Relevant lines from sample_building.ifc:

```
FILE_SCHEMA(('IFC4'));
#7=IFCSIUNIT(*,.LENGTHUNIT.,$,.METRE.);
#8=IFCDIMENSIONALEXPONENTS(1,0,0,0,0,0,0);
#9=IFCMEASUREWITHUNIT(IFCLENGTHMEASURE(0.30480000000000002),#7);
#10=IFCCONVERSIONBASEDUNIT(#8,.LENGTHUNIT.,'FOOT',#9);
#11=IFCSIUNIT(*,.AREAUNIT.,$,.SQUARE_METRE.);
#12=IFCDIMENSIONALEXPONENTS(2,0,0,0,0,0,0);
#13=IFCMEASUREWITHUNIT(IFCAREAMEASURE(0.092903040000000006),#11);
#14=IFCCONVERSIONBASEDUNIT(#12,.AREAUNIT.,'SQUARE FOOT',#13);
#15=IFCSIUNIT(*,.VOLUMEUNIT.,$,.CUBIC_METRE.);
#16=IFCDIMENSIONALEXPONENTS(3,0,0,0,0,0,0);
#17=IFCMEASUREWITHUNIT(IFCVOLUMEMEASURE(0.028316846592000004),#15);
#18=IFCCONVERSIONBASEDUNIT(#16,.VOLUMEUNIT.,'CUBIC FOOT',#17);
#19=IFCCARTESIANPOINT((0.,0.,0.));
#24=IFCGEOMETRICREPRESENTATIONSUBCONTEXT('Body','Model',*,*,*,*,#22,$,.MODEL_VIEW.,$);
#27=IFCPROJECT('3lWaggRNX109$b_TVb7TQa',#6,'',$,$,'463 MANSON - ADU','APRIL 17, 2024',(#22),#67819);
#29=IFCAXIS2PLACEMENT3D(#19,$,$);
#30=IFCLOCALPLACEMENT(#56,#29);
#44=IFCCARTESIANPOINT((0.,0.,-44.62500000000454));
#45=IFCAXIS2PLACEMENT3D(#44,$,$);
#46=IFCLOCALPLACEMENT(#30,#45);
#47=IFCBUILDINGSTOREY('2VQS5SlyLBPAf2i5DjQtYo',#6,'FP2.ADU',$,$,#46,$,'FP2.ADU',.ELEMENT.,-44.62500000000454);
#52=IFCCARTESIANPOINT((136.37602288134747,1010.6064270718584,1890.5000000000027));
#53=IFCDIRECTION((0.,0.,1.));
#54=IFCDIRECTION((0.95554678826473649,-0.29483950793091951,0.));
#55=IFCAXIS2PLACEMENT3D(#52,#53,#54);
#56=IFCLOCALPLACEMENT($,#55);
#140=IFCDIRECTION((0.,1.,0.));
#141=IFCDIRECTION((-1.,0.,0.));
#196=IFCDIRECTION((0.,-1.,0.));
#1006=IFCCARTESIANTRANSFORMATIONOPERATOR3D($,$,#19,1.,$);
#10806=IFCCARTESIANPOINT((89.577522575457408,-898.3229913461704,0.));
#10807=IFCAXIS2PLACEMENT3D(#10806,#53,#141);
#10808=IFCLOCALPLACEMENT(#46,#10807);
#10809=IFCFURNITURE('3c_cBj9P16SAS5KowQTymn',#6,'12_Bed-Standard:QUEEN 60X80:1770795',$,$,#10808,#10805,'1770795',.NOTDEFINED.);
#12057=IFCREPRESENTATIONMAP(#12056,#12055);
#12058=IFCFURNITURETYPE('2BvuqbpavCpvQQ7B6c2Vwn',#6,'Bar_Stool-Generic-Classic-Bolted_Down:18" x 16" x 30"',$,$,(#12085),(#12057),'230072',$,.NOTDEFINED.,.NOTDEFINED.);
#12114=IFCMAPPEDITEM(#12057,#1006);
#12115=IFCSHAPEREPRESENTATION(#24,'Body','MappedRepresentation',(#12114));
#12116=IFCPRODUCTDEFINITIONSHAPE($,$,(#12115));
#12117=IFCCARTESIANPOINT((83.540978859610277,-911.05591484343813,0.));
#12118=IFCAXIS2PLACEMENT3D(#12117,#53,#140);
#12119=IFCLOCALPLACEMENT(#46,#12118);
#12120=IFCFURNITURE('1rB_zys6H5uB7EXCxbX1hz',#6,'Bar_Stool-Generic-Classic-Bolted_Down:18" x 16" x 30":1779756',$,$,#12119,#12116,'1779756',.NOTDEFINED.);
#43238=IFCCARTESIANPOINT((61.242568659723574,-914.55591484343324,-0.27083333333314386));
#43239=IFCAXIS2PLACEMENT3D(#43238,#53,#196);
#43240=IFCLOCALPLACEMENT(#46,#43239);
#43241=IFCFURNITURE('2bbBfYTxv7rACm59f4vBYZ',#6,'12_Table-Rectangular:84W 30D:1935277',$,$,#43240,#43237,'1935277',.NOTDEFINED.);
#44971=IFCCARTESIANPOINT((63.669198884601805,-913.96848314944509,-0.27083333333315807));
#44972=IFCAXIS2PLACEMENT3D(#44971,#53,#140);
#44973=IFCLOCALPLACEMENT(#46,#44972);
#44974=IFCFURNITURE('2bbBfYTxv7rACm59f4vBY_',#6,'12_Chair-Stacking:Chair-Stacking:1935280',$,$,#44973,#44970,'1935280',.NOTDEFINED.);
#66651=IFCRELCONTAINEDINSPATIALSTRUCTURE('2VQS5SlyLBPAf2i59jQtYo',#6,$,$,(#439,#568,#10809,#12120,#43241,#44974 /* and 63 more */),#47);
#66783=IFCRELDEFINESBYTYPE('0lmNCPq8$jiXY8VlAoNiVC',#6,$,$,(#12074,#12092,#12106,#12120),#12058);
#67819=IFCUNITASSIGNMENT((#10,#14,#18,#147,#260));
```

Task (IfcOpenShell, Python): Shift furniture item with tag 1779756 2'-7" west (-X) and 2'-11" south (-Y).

```python
import ifcopenshell
import ifcopenshell.api.geometry
import ifcopenshell.util.placement
import ifcopenshell.util.unit

model = ifcopenshell.open("sample_building.ifc")
unit_scale = ifcopenshell.util.unit.calculate_unit_scale(model)

item = model.by_guid("1rB_zys6H5uB7EXCxbX1hz")
matrix = ifcopenshell.util.placement.get_local_placement(item.ObjectPlacement)
matrix[0, 3] -= 31 * 0.0254 / unit_scale
matrix[1, 3] -= 35 * 0.0254 / unit_scale
ifcopenshell.api.geometry.edit_object_placement(model, product=item, matrix=matrix, is_si=False)

print(ifcopenshell.util.placement.get_local_placement(item.ObjectPlacement).round(3) + 0.0)

model.write("sample_building_edited.ifc")
```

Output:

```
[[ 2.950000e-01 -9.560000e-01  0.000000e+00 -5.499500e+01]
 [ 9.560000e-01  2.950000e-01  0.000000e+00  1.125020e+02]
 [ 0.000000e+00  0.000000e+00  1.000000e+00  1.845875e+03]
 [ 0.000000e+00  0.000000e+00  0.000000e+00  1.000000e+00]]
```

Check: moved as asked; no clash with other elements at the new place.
